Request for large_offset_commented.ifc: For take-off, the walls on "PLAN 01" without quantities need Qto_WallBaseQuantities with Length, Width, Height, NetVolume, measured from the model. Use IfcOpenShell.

First a look at what the model holds.

```python
import ifcopenshell
import ifcopenshell.util.element
import ifcopenshell.util.unit

model = ifcopenshell.open("large_offset_commented.ifc")
print(model.schema)
for unit_type in ("LENGTHUNIT", "AREAUNIT", "VOLUMEUNIT"):
    print(unit_type, ifcopenshell.util.unit.calculate_unit_scale(model, unit_type))
storey = next(s for s in model.by_type("IfcBuildingStorey") if s.Name == "PLAN 01")
walls = [e for e in ifcopenshell.util.element.get_decomposition(storey) if e.is_a("IfcWall")]
for e in sorted(walls, key=lambda e: e.id()):
    print(e.id(), e.is_a(), e.Name, list(ifcopenshell.util.element.get_psets(e, qtos_only=True)), sep=" | ")
```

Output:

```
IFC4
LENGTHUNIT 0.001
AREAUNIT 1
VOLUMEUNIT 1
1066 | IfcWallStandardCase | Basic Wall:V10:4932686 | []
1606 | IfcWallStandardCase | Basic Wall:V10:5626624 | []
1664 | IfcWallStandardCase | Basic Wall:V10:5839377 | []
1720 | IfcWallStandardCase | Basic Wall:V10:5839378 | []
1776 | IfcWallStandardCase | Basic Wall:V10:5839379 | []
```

```python
import ifcopenshell
import ifcopenshell.api.pset
import ifcopenshell.geom
import ifcopenshell.util.element
import ifcopenshell.util.shape
import ifcopenshell.util.unit

model = ifcopenshell.open("large_offset_commented.ifc")
unit_scale = ifcopenshell.util.unit.calculate_unit_scale(model)
volume_scale = ifcopenshell.util.unit.calculate_unit_scale(model, "VOLUMEUNIT")
settings = ifcopenshell.geom.settings()

storey = next(s for s in model.by_type("IfcBuildingStorey") if s.Name == "PLAN 01")
walls = [e for e in ifcopenshell.util.element.get_decomposition(storey) if e.is_a("IfcWall")]

for e in sorted(walls, key=lambda e: e.id()):
    if ifcopenshell.util.element.get_psets(e, qtos_only=True, should_inherit=False):
        continue
    # Geometry comes back in metres, in the element's own axes.
    shape = ifcopenshell.geom.create_shape(settings, e)
    values = {
        "Length": ifcopenshell.util.shape.get_x(shape.geometry) / unit_scale,
        "Width": ifcopenshell.util.shape.get_y(shape.geometry) / unit_scale,
        "Height": ifcopenshell.util.shape.get_z(shape.geometry) / unit_scale,
        "NetVolume": ifcopenshell.util.shape.get_volume(shape.geometry) / volume_scale,
    }
    qto = ifcopenshell.api.pset.add_qto(model, product=e, name="Qto_WallBaseQuantities")
    ifcopenshell.api.pset.edit_qto(model, qto=qto, properties=values)
    print(e.id(), {k: round(v, 3) for k, v in values.items()})

model.write("large_offset_commented_v2.ifc")
```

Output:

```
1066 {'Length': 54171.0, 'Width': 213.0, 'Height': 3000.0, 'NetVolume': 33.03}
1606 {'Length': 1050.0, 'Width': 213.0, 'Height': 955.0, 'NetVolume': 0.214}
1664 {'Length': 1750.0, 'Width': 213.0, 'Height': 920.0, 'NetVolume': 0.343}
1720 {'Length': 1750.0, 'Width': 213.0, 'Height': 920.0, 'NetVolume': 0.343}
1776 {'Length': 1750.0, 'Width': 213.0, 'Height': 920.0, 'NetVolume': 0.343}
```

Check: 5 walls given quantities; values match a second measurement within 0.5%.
